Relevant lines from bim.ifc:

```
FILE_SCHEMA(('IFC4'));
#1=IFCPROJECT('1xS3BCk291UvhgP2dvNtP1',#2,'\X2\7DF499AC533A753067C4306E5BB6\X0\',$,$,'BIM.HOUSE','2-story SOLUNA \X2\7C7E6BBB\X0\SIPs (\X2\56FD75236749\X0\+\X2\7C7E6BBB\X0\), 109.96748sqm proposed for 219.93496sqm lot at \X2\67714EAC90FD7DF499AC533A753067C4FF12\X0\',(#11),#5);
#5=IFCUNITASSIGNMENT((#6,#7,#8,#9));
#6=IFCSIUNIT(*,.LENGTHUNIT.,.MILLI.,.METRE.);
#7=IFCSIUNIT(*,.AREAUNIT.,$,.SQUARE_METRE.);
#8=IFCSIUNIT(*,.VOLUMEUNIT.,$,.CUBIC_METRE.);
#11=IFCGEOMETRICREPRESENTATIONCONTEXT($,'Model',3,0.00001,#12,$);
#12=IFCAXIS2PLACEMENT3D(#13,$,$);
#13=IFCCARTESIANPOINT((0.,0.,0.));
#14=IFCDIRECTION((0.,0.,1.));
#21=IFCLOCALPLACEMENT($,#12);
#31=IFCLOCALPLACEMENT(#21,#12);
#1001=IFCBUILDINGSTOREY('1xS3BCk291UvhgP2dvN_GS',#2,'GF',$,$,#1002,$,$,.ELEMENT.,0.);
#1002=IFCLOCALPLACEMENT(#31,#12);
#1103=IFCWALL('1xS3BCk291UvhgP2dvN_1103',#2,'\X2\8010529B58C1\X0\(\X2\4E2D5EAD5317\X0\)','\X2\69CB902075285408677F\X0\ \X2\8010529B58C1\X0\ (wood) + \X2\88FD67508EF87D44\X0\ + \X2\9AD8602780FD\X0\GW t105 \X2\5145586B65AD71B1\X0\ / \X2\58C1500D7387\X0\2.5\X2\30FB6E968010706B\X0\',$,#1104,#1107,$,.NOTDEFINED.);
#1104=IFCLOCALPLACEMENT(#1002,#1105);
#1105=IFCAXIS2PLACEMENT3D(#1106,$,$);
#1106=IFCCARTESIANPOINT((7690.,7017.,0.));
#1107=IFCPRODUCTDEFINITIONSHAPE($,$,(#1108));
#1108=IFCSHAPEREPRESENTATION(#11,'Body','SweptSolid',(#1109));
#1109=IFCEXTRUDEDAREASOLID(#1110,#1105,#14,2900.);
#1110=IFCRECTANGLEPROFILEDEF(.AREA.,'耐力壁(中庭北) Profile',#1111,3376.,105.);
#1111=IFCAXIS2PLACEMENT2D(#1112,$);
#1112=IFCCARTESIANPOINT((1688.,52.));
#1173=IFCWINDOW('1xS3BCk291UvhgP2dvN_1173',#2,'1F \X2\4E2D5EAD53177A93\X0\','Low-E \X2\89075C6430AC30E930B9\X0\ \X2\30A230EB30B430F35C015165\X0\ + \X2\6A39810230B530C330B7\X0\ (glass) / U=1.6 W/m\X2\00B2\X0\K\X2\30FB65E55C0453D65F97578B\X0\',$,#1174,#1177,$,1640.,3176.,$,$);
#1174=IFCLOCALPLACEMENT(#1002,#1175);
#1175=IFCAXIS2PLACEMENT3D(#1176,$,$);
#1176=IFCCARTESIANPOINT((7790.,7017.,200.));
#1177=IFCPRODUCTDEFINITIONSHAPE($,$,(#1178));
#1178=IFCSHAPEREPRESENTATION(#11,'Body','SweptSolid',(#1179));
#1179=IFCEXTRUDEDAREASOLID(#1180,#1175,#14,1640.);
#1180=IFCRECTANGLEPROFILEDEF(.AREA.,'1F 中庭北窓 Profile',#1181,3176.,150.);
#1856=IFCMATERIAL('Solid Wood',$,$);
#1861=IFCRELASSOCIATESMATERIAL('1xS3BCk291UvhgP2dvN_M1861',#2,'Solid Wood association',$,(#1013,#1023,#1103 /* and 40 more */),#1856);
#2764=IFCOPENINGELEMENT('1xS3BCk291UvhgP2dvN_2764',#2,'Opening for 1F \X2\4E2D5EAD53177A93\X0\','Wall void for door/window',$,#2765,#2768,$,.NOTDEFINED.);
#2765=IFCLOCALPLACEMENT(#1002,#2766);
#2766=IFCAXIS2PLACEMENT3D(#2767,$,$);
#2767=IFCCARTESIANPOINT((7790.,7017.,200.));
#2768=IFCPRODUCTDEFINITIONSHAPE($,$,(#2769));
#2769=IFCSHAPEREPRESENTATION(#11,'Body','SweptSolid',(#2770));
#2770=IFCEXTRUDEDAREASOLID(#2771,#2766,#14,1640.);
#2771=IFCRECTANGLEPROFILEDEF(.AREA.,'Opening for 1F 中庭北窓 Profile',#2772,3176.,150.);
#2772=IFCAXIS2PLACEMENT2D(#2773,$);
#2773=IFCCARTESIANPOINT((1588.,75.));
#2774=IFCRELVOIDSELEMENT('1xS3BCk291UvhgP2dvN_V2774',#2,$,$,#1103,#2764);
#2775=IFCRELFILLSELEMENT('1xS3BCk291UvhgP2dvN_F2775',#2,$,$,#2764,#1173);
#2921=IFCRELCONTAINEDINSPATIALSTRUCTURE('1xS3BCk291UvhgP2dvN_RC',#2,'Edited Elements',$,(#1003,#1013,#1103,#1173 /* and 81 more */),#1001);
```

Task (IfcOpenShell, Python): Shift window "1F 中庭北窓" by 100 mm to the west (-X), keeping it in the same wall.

```python
import ifcopenshell
import ifcopenshell.api.geometry
import ifcopenshell.util.placement
import ifcopenshell.util.unit

model = ifcopenshell.open("bim.ifc")
unit_scale = ifcopenshell.util.unit.calculate_unit_scale(model)

window = model.by_id(1173)
opening = window.FillsVoids[0].RelatingOpeningElement
wall = opening.VoidsElements[0].RelatingBuildingElement

wall_matrix = ifcopenshell.util.placement.get_local_placement(wall.ObjectPlacement)
shift = wall_matrix[:3, 0] * -0.1 / unit_scale
before = ifcopenshell.util.placement.get_local_placement(window.ObjectPlacement)[:3, 3].copy()

# The window is not placed relative to its opening, so move both.
for product in (opening, window):
    matrix = ifcopenshell.util.placement.get_local_placement(product.ObjectPlacement)
    matrix[:3, 3] += shift
    ifcopenshell.api.geometry.edit_object_placement(model, product=product, matrix=matrix, is_si=False)

after = ifcopenshell.util.placement.get_local_placement(window.ObjectPlacement)[:3, 3]
print("window moved by", (after - before).round(3) + 0.0)

model.write("bim-out.ifc")
```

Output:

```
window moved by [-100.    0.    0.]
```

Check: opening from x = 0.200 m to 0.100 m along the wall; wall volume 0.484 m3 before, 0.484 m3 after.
